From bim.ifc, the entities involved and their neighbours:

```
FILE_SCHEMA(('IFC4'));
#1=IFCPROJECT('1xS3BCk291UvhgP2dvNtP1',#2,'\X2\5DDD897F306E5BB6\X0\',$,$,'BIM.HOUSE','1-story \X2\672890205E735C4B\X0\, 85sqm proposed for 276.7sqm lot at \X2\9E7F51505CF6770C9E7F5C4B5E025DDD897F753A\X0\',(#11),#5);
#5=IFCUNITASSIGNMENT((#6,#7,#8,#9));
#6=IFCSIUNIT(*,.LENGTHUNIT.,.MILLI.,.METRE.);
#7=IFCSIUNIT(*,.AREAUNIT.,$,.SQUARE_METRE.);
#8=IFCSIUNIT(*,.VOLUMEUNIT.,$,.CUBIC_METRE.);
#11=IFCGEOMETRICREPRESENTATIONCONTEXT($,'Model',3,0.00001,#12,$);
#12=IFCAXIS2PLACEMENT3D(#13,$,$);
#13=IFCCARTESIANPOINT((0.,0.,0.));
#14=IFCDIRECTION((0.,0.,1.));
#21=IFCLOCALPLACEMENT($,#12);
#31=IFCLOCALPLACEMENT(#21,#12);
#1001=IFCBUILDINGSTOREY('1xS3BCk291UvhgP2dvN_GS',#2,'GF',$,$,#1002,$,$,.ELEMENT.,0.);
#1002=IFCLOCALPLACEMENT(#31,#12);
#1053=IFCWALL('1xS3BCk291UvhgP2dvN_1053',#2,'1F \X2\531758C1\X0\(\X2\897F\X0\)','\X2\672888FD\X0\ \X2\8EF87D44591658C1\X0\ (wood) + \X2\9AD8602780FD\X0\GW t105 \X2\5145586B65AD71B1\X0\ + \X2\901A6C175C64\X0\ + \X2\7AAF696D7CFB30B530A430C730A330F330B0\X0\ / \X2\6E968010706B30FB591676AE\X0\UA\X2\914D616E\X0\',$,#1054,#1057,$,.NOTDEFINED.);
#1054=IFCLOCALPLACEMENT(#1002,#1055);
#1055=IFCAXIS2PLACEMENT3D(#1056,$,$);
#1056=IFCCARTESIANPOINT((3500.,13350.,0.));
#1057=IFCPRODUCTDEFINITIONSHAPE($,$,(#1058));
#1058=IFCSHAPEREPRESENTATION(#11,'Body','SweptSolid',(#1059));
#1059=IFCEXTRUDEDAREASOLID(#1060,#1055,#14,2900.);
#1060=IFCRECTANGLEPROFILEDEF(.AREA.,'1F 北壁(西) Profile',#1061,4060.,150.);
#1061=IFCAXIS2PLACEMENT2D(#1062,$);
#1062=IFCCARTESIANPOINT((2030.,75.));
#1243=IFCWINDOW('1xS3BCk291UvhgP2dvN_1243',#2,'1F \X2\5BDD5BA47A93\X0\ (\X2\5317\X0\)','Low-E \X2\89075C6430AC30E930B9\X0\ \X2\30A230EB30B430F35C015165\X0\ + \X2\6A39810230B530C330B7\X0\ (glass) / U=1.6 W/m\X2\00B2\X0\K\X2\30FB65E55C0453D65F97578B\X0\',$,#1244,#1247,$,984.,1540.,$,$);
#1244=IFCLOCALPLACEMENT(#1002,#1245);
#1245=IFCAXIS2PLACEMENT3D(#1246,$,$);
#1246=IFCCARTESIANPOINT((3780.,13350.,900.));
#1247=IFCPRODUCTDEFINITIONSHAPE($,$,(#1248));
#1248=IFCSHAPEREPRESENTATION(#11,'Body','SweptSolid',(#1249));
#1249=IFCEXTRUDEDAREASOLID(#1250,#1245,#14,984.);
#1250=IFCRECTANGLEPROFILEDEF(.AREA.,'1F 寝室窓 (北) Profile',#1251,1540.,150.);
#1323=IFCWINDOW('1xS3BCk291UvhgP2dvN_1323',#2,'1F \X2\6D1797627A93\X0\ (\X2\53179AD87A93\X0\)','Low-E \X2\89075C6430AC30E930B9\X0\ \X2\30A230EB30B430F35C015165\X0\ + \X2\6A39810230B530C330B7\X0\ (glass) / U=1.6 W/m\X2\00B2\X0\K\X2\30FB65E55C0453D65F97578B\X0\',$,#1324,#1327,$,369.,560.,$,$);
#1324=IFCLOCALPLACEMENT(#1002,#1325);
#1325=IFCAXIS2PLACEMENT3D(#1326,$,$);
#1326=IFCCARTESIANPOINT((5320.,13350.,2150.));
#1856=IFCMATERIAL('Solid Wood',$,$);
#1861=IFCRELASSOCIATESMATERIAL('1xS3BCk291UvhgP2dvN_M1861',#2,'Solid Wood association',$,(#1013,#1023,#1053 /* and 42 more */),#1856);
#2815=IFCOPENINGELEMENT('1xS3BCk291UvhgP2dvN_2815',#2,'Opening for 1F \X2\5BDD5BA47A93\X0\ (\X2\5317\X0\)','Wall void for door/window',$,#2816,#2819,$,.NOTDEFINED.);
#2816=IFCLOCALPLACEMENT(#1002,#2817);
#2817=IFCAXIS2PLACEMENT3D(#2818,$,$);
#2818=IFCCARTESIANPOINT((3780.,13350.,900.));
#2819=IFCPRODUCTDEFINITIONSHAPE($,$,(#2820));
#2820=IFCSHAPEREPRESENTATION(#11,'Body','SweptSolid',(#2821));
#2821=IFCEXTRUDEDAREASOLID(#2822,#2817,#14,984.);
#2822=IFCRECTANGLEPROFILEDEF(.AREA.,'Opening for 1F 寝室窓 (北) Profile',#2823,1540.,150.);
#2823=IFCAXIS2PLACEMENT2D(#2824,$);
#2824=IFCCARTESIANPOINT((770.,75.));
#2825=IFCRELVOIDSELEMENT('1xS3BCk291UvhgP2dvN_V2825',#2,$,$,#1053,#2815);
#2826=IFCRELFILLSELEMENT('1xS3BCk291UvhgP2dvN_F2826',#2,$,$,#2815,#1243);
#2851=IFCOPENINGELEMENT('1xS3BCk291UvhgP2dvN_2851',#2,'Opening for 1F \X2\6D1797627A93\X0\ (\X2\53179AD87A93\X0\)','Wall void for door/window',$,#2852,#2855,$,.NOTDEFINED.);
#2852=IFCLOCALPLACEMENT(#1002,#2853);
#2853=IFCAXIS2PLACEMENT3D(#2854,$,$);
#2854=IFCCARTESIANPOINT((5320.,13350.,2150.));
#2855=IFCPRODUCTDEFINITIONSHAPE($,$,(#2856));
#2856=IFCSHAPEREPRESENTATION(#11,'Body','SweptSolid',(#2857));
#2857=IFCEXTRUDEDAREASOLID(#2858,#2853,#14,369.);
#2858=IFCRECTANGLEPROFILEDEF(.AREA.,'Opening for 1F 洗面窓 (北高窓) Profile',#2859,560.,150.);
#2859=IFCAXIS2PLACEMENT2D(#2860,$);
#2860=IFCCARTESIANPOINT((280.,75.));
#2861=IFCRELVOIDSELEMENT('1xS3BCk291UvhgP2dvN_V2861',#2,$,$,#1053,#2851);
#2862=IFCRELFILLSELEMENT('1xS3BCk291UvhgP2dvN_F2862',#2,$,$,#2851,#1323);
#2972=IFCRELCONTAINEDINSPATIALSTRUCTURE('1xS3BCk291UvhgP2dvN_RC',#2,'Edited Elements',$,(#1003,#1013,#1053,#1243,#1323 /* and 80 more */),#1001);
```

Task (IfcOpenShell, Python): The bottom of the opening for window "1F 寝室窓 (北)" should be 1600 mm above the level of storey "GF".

```python
import numpy as np
import ifcopenshell
import ifcopenshell.api.geometry
import ifcopenshell.geom
import ifcopenshell.util.element
import ifcopenshell.util.placement
import ifcopenshell.util.shape
import ifcopenshell.util.unit

model = ifcopenshell.open("bim.ifc")
unit_scale = ifcopenshell.util.unit.calculate_unit_scale(model)

window = model.by_guid("1xS3BCk291UvhgP2dvN_1243")
opening = window.FillsVoids[0].RelatingOpeningElement
storey = ifcopenshell.util.element.get_container(window, ifc_class="IfcBuildingStorey")
level = ifcopenshell.util.placement.get_local_placement(storey.ObjectPlacement)[2, 3]

# The opening's origin need not be at the sill, so measure its lowest point.
shape = ifcopenshell.geom.create_shape(ifcopenshell.geom.settings(), opening)
bottom = ifcopenshell.util.shape.get_shape_bottom_elevation(shape, shape.geometry) / unit_scale
dz = level + 1600.0 - bottom

shift = np.array([0.0, 0.0, dz])
# The window is not placed relative to its opening, so move both.
for product in (opening, window):
    matrix = ifcopenshell.util.placement.get_local_placement(product.ObjectPlacement)
    matrix[:3, 3] += shift
    ifcopenshell.api.geometry.edit_object_placement(model, product=product, matrix=matrix, is_si=False)

print(f"moved by {dz * unit_scale:+.3f} m")

model.write("bim_v2.ifc")
```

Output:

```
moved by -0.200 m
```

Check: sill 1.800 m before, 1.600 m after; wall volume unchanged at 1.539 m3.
